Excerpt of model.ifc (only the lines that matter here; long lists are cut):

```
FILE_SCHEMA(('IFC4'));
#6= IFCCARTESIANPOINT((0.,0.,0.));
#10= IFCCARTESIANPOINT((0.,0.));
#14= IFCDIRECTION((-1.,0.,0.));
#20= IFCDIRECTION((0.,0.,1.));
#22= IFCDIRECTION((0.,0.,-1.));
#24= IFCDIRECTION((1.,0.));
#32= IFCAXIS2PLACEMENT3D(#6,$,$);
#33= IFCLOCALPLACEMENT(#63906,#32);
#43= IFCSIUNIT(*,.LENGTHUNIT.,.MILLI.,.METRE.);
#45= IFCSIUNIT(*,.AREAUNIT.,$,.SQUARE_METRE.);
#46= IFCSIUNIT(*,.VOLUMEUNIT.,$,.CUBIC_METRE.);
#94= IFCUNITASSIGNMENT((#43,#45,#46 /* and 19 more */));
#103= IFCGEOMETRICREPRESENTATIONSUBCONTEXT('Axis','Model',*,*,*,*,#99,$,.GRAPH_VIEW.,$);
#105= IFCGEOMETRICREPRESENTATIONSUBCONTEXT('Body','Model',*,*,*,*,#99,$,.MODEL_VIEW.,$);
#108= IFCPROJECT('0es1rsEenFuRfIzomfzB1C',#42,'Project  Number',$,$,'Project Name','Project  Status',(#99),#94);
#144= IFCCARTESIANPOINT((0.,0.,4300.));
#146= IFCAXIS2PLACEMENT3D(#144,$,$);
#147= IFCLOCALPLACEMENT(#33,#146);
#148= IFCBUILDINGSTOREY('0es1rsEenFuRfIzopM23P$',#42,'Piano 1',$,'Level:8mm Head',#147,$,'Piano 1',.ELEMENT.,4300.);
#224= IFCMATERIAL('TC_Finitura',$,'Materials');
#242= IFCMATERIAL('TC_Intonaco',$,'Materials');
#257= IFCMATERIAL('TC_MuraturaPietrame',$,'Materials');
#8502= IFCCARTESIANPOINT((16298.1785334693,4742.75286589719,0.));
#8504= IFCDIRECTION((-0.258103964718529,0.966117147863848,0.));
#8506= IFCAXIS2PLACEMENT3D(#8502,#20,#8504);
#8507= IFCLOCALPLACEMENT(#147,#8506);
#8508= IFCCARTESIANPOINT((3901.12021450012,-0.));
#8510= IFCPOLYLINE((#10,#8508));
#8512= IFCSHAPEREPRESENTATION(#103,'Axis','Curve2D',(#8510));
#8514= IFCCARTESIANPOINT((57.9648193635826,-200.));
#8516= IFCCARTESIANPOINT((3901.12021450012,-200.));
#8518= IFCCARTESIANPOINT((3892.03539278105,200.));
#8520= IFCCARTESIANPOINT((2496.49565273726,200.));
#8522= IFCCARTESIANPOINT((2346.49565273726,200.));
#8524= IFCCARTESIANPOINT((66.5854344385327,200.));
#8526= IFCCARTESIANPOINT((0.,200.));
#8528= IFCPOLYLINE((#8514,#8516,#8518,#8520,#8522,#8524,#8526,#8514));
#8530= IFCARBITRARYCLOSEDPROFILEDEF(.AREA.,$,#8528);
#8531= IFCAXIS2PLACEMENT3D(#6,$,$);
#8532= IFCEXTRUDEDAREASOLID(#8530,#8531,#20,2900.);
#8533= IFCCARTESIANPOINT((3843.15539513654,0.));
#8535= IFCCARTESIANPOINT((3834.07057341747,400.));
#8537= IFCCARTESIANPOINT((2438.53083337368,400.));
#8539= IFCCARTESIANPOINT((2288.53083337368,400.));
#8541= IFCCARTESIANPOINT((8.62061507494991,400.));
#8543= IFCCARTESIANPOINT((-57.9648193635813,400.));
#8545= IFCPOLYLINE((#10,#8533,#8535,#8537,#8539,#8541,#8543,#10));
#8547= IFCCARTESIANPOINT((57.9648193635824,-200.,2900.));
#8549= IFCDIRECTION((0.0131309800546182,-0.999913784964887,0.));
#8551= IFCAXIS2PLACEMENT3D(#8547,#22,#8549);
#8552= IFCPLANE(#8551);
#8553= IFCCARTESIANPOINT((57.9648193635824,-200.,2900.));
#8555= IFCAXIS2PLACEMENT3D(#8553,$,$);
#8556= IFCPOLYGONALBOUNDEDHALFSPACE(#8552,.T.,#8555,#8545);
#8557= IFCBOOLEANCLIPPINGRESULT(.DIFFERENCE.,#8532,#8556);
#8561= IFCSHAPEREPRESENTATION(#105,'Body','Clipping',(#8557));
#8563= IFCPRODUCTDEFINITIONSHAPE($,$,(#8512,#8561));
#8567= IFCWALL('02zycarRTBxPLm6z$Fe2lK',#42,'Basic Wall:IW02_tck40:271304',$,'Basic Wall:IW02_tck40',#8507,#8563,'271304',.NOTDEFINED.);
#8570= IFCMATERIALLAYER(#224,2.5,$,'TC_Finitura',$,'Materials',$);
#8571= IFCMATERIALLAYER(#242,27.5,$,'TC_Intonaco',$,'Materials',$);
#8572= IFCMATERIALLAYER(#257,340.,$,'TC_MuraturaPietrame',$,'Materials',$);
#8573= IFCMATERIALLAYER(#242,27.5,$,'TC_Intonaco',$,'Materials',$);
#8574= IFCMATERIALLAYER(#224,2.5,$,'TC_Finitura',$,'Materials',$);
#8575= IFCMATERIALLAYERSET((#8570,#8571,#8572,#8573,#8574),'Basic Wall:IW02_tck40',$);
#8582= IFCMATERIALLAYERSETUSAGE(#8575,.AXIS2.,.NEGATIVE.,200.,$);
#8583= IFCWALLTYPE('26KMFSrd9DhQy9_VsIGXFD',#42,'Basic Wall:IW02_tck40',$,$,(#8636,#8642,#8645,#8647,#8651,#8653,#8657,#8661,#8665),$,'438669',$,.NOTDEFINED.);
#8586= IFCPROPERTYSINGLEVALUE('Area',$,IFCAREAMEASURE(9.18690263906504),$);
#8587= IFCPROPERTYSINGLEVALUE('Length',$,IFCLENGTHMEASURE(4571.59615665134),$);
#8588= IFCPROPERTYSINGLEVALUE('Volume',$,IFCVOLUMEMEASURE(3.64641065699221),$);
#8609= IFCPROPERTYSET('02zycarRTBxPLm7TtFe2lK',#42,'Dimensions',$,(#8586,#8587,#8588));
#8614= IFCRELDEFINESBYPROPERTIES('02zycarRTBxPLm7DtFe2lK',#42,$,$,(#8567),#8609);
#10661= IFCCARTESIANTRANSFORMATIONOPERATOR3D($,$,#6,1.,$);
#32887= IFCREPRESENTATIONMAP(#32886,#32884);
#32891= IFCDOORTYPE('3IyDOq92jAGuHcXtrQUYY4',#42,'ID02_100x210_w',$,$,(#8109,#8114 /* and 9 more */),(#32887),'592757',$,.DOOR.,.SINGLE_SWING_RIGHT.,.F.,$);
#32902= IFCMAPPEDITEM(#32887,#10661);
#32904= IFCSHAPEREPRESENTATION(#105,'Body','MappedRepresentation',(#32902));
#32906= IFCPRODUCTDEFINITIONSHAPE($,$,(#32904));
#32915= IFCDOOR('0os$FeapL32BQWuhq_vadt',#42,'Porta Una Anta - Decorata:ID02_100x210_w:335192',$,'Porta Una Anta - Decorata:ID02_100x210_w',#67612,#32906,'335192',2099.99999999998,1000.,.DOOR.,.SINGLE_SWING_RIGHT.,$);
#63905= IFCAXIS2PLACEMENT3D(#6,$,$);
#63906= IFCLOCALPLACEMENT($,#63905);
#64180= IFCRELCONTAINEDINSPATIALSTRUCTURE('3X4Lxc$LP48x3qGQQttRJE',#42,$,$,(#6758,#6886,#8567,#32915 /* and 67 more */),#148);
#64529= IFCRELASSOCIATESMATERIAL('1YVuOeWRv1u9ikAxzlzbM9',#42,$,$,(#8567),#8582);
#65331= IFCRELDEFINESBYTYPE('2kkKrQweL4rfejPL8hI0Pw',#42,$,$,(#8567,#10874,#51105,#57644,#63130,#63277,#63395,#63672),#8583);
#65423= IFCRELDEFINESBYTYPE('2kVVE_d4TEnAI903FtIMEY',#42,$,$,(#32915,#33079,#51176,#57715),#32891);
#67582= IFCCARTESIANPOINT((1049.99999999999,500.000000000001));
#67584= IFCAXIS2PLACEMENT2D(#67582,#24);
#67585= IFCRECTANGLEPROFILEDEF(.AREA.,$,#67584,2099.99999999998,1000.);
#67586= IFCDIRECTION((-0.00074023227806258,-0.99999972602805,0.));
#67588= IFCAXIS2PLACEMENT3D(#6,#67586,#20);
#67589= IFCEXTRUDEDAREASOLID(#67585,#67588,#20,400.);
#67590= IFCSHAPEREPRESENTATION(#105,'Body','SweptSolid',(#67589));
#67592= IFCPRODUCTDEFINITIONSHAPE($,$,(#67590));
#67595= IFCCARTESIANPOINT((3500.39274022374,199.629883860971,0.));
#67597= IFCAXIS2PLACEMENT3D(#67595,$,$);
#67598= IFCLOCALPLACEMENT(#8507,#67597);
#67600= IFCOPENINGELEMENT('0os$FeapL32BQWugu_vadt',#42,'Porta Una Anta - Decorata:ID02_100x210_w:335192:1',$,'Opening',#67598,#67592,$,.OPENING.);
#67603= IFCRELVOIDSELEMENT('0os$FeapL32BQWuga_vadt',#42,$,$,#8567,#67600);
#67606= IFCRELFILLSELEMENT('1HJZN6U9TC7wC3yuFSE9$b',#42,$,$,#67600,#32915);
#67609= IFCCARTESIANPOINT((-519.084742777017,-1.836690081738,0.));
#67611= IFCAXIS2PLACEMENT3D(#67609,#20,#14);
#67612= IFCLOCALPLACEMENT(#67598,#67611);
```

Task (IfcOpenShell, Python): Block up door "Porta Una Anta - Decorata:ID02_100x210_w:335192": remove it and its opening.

```python
import ifcopenshell
import ifcopenshell.api.feature
import ifcopenshell.api.pset
import ifcopenshell.api.root
import ifcopenshell.geom
import ifcopenshell.util.element
import ifcopenshell.util.shape
import ifcopenshell.util.unit

model = ifcopenshell.open("model.ifc")
area_scale = ifcopenshell.util.unit.calculate_unit_scale(model, "AREAUNIT")
volume_scale = ifcopenshell.util.unit.calculate_unit_scale(model, "VOLUMEUNIT")
settings = ifcopenshell.geom.settings()


def volume(element):
    """Net volume in cubic metres, openings subtracted."""
    shape = ifcopenshell.geom.create_shape(settings, element)
    return ifcopenshell.util.shape.get_volume(shape.geometry)


door = model.by_id(32915)
opening = door.FillsVoids[0].RelatingOpeningElement
wall = opening.VoidsElements[0].RelatingBuildingElement
before = volume(wall)

ifcopenshell.api.root.remove_product(model, product=door)
ifcopenshell.api.feature.remove_feature(model, feature=opening)

after = volume(wall)
thickness = 0.4  # wall thickness in metres

# Update the wall's stored quantities.
pset = model.by_id(ifcopenshell.util.element.get_pset(wall, "Dimensions", should_inherit=False)["id"])
ifcopenshell.api.pset.edit_pset(model, pset=pset, properties={
    "Area": model.create_entity("IfcAreaMeasure", after / thickness / area_scale),
    "Volume": model.create_entity("IfcVolumeMeasure", after / volume_scale),
})

print(f"wall volume {before:.3f} -> {after:.3f} m3")

model.write("model_updated.ifc")
```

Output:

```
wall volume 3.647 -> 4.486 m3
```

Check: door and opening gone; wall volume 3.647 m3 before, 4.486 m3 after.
